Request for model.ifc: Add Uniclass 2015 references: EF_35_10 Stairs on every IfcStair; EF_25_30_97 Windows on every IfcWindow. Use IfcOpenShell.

First a look at what the model holds.

```python
import ifcopenshell

model = ifcopenshell.open("model.ifc")
print(model.schema)
print("classifications:", [c.Name for c in model.by_type("IfcClassification")])
for ifc_class in ("IfcDoor", "IfcRoof", "IfcStair", "IfcWall", "IfcWindow"):
    print(ifc_class, len(model.by_type(ifc_class)))
```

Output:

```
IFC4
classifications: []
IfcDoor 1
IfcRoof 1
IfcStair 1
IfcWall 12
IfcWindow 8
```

```python
import ifcopenshell
import ifcopenshell.api.classification

model = ifcopenshell.open("model.ifc")

system = ifcopenshell.api.classification.add_classification(model, classification="Uniclass 2015")

codes = {
    "IfcStair": ("EF_35_10", "Stairs"),
    "IfcWindow": ("EF_25_30_97", "Windows"),
}
for ifc_class, (code, name) in codes.items():
    products = model.by_type(ifc_class)
    ifcopenshell.api.classification.add_reference(
        model, products=products, classification=system, identification=code, name=name
    )
    print(code, len(products))

model.write("model-out.ifc")
```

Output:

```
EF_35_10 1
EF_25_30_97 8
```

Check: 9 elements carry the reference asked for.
